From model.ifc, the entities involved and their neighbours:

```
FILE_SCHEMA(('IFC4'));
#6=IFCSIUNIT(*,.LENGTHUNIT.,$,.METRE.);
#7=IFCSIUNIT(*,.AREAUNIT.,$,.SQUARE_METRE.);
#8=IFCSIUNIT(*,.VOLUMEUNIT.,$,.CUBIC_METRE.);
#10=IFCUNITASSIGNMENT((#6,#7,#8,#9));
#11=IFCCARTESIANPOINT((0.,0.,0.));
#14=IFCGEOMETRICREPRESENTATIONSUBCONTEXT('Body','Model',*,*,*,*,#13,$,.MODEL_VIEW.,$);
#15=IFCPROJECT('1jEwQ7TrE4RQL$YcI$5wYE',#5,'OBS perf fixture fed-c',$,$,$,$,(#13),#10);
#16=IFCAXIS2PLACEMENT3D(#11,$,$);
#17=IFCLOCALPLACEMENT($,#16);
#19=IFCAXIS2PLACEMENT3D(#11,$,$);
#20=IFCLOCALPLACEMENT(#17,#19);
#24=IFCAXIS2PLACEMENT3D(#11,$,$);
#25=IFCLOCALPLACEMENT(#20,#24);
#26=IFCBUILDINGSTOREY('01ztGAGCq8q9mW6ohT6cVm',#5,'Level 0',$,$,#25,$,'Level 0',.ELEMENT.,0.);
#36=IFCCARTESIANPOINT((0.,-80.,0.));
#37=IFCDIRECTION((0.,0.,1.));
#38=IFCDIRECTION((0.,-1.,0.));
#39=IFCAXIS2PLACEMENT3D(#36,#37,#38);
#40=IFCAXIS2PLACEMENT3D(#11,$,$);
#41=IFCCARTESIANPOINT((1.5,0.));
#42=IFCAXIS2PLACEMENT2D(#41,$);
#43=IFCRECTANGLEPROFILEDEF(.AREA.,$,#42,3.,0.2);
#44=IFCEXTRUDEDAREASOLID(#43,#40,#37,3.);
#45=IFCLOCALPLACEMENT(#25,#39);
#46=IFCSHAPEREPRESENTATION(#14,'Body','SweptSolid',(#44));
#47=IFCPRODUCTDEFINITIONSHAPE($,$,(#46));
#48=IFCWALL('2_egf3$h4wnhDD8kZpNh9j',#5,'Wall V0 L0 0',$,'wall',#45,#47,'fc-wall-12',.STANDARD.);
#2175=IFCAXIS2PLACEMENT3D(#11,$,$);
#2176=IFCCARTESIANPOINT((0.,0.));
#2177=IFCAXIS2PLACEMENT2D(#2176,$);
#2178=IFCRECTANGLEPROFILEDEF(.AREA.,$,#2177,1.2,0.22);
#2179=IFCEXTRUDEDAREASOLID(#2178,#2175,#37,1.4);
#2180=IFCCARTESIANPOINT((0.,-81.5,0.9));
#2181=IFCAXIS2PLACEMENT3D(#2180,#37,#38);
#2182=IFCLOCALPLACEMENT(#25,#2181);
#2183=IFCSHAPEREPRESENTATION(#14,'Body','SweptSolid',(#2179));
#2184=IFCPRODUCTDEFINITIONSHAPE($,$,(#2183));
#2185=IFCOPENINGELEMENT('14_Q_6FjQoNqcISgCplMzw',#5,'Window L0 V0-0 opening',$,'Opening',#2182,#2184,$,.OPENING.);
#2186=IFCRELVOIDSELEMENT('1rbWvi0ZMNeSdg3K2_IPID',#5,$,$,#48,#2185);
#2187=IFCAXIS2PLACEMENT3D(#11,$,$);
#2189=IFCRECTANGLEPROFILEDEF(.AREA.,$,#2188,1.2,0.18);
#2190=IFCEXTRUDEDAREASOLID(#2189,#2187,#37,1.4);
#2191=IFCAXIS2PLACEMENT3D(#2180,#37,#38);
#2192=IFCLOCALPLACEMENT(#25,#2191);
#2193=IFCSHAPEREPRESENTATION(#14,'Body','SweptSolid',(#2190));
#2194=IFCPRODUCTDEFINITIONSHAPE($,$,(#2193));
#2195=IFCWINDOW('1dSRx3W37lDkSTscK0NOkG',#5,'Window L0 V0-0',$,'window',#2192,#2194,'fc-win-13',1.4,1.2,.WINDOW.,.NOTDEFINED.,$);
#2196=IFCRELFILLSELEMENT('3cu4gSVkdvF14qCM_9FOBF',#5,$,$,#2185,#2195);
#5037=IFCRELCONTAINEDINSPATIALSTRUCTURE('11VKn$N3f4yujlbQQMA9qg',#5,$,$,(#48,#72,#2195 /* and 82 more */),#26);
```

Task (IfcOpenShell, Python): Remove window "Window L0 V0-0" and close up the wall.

```python
import ifcopenshell
import ifcopenshell.api.feature
import ifcopenshell.api.root
import ifcopenshell.geom
import ifcopenshell.util.shape

model = ifcopenshell.open("model.ifc")
settings = ifcopenshell.geom.settings()


def volume(element):
    """Net volume in cubic metres, openings subtracted."""
    shape = ifcopenshell.geom.create_shape(settings, element)
    return ifcopenshell.util.shape.get_volume(shape.geometry)


window = model.by_guid("1dSRx3W37lDkSTscK0NOkG")
opening = window.FillsVoids[0].RelatingOpeningElement
wall = opening.VoidsElements[0].RelatingBuildingElement
before = volume(wall)

ifcopenshell.api.root.remove_product(model, product=window)
ifcopenshell.api.feature.remove_feature(model, feature=opening)

after = volume(wall)

print(f"wall volume {before:.3f} -> {after:.3f} m3")

model.write("model_v2.ifc")
```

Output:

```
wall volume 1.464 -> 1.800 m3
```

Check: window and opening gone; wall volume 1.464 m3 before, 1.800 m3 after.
